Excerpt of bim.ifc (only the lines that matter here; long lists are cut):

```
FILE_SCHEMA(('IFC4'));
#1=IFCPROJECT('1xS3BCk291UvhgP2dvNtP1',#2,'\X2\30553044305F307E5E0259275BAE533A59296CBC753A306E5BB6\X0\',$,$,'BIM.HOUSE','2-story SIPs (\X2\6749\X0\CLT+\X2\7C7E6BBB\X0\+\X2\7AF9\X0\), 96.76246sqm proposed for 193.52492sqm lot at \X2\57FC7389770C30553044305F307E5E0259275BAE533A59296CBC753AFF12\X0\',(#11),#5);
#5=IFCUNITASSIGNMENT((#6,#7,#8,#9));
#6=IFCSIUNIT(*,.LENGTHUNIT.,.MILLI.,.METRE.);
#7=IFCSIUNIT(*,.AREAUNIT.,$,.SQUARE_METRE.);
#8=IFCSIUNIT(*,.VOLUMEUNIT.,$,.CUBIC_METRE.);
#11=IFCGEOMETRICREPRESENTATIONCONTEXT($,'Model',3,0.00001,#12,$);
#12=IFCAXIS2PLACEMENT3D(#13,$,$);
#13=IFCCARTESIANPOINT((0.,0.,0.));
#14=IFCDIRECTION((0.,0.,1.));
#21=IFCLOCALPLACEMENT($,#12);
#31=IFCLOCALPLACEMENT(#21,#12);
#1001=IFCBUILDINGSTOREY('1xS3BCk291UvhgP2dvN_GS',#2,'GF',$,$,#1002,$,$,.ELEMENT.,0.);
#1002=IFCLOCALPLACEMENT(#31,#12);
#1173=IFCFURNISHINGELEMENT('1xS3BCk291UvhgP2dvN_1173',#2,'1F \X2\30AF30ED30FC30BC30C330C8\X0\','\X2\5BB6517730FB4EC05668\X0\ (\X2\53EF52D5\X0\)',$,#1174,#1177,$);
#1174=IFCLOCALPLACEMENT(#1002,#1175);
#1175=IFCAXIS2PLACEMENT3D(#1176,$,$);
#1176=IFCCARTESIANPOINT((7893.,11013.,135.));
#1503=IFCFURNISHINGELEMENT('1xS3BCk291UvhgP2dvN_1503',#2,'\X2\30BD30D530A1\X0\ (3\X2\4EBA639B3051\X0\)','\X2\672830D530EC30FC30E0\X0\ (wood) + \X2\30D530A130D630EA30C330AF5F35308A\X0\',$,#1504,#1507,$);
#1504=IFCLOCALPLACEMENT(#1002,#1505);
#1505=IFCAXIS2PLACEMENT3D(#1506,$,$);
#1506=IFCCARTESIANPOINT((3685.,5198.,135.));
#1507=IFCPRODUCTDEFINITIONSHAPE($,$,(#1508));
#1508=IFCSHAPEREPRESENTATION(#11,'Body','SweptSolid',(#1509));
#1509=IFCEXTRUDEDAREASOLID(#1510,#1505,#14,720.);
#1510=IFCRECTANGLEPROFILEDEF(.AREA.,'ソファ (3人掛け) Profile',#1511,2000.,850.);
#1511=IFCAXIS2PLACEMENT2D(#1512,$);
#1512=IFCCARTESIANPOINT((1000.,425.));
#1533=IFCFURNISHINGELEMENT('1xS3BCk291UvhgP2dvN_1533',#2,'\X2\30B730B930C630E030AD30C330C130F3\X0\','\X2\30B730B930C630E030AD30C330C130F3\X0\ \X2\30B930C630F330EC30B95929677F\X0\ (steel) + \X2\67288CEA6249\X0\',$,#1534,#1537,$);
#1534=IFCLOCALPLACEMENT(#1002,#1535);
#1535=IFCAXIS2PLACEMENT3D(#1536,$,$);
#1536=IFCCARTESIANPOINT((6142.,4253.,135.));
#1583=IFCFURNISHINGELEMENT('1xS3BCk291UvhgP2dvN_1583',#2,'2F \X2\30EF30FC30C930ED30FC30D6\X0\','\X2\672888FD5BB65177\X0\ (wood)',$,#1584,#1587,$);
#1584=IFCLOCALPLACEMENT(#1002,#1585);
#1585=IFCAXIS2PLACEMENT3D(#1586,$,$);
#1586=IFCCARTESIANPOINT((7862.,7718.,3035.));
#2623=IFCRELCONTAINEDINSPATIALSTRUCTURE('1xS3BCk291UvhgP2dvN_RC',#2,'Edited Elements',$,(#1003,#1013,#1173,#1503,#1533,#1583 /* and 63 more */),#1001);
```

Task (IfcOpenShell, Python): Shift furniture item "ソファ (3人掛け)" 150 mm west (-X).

```python
import ifcopenshell
import ifcopenshell.api.geometry
import ifcopenshell.util.placement

model = ifcopenshell.open("bim.ifc")

item = model.by_id(1503)
matrix = ifcopenshell.util.placement.get_local_placement(item.ObjectPlacement)
matrix[0, 3] -= 150.0
ifcopenshell.api.geometry.edit_object_placement(model, product=item, matrix=matrix, is_si=False)

print(ifcopenshell.util.placement.get_local_placement(item.ObjectPlacement).round(3) + 0.0)

model.write("bim_v2.ifc")
```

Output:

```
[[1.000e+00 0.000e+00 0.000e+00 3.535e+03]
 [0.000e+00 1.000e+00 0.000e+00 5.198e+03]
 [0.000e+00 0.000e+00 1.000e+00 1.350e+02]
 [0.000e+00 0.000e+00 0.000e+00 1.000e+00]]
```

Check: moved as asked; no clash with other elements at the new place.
